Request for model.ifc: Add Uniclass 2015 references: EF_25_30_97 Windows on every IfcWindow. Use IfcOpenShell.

First a look at what the model holds.

```python
import ifcopenshell

model = ifcopenshell.open("model.ifc")
print(model.schema)
print("classifications:", [c.Name for c in model.by_type("IfcClassification")])
for ifc_class in ("IfcDoor", "IfcRoof", "IfcStair", "IfcWall", "IfcWindow"):
    print(ifc_class, len(model.by_type(ifc_class)))
```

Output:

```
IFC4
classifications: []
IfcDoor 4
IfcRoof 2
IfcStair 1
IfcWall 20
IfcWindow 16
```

```python
import ifcopenshell
import ifcopenshell.api.classification

model = ifcopenshell.open("model.ifc")

system = ifcopenshell.api.classification.add_classification(model, classification="Uniclass 2015")

codes = {
    "IfcWindow": ("EF_25_30_97", "Windows"),
}
for ifc_class, (code, name) in codes.items():
    products = model.by_type(ifc_class)
    ifcopenshell.api.classification.add_reference(
        model, products=products, classification=system, identification=code, name=name
    )
    print(code, len(products))

model.write("model_v2.ifc")
```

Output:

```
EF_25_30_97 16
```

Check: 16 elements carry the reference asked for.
